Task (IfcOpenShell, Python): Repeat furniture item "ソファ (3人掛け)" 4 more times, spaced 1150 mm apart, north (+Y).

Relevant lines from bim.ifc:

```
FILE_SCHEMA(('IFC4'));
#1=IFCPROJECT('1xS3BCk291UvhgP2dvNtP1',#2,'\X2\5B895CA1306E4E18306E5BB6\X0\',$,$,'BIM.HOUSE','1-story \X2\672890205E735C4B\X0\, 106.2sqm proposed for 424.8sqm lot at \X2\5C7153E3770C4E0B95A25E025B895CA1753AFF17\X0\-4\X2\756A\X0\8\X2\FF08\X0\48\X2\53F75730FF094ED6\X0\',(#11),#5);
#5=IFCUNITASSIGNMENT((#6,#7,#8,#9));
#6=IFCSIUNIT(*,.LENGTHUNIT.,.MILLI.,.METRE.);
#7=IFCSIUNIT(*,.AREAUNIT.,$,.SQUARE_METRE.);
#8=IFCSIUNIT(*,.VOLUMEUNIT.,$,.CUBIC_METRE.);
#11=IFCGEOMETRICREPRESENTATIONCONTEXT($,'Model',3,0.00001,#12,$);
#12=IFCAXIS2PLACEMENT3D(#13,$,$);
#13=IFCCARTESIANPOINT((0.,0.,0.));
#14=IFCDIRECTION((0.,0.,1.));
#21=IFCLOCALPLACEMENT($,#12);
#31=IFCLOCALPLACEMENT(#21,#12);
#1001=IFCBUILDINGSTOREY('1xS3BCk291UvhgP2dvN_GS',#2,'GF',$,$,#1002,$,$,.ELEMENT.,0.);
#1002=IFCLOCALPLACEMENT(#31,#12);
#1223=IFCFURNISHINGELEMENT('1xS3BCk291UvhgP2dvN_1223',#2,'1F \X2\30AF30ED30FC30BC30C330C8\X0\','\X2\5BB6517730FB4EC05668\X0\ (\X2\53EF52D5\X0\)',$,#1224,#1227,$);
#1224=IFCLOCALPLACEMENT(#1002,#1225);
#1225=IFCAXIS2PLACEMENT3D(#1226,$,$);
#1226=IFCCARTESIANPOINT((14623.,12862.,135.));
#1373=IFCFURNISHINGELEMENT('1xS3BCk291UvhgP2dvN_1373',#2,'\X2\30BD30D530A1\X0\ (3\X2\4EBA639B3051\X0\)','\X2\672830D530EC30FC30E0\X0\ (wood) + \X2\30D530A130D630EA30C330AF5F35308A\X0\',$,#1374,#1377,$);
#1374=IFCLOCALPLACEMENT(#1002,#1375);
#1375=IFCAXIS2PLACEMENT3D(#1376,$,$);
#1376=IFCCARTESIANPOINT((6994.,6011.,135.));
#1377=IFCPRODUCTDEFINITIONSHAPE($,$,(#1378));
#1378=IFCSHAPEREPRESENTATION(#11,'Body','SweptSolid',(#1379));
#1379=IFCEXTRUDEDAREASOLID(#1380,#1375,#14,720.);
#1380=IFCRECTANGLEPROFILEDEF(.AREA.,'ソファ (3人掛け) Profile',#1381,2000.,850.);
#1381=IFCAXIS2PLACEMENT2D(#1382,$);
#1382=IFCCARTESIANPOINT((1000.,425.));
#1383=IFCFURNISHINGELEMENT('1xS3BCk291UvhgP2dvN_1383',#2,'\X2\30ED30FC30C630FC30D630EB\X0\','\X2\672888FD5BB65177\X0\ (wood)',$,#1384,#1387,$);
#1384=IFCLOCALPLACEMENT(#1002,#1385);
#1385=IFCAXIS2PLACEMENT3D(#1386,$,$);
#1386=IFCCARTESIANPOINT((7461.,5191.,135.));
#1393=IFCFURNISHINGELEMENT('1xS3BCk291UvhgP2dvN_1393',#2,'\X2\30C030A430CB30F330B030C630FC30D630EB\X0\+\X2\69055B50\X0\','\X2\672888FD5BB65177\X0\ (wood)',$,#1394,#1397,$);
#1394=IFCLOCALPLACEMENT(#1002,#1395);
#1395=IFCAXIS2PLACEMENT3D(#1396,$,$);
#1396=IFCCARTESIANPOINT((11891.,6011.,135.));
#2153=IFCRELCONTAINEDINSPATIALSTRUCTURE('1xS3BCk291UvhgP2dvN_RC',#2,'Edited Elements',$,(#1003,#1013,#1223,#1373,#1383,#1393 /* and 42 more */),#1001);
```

```python
import numpy as np
import ifcopenshell
import ifcopenshell.api.geometry
import ifcopenshell.api.root
import ifcopenshell.util.element
import ifcopenshell.util.placement

model = ifcopenshell.open("bim.ifc")


def reuse_history(source, copy):
    """copy_class also copies each property set's owner history, people and application; keep the originals."""
    for rel in copy.IsDefinedBy:
        if rel.is_a("IfcRelDefinesByProperties") and (history := rel.RelatingPropertyDefinition.OwnerHistory):
            rel.RelatingPropertyDefinition.OwnerHistory = source.OwnerHistory
            ifcopenshell.util.element.remove_deep2(model, history)


source = model.by_guid("1xS3BCk291UvhgP2dvN_1373")
base = ifcopenshell.util.placement.get_local_placement(source.ObjectPlacement)
step = np.array([0.0, 1.0, 0.0]) * 1150.0

for i in range(1, 5):
    copy = ifcopenshell.api.root.copy_class(model, product=source)
    copy.Representation = ifcopenshell.util.element.copy_deep(
        model, source.Representation, exclude=["IfcGeometricRepresentationContext", "IfcRepresentationMap"]
    )
    reuse_history(source, copy)
    matrix = base.copy()
    matrix[:3, 3] += i * step
    print("added at", matrix[:3, 3].round(3) + 0.0)
    ifcopenshell.api.geometry.edit_object_placement(model, product=copy, matrix=matrix, is_si=False)

model.write("bim_v2.ifc")
```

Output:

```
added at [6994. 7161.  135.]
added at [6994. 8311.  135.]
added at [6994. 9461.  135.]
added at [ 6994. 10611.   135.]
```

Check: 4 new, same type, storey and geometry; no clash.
